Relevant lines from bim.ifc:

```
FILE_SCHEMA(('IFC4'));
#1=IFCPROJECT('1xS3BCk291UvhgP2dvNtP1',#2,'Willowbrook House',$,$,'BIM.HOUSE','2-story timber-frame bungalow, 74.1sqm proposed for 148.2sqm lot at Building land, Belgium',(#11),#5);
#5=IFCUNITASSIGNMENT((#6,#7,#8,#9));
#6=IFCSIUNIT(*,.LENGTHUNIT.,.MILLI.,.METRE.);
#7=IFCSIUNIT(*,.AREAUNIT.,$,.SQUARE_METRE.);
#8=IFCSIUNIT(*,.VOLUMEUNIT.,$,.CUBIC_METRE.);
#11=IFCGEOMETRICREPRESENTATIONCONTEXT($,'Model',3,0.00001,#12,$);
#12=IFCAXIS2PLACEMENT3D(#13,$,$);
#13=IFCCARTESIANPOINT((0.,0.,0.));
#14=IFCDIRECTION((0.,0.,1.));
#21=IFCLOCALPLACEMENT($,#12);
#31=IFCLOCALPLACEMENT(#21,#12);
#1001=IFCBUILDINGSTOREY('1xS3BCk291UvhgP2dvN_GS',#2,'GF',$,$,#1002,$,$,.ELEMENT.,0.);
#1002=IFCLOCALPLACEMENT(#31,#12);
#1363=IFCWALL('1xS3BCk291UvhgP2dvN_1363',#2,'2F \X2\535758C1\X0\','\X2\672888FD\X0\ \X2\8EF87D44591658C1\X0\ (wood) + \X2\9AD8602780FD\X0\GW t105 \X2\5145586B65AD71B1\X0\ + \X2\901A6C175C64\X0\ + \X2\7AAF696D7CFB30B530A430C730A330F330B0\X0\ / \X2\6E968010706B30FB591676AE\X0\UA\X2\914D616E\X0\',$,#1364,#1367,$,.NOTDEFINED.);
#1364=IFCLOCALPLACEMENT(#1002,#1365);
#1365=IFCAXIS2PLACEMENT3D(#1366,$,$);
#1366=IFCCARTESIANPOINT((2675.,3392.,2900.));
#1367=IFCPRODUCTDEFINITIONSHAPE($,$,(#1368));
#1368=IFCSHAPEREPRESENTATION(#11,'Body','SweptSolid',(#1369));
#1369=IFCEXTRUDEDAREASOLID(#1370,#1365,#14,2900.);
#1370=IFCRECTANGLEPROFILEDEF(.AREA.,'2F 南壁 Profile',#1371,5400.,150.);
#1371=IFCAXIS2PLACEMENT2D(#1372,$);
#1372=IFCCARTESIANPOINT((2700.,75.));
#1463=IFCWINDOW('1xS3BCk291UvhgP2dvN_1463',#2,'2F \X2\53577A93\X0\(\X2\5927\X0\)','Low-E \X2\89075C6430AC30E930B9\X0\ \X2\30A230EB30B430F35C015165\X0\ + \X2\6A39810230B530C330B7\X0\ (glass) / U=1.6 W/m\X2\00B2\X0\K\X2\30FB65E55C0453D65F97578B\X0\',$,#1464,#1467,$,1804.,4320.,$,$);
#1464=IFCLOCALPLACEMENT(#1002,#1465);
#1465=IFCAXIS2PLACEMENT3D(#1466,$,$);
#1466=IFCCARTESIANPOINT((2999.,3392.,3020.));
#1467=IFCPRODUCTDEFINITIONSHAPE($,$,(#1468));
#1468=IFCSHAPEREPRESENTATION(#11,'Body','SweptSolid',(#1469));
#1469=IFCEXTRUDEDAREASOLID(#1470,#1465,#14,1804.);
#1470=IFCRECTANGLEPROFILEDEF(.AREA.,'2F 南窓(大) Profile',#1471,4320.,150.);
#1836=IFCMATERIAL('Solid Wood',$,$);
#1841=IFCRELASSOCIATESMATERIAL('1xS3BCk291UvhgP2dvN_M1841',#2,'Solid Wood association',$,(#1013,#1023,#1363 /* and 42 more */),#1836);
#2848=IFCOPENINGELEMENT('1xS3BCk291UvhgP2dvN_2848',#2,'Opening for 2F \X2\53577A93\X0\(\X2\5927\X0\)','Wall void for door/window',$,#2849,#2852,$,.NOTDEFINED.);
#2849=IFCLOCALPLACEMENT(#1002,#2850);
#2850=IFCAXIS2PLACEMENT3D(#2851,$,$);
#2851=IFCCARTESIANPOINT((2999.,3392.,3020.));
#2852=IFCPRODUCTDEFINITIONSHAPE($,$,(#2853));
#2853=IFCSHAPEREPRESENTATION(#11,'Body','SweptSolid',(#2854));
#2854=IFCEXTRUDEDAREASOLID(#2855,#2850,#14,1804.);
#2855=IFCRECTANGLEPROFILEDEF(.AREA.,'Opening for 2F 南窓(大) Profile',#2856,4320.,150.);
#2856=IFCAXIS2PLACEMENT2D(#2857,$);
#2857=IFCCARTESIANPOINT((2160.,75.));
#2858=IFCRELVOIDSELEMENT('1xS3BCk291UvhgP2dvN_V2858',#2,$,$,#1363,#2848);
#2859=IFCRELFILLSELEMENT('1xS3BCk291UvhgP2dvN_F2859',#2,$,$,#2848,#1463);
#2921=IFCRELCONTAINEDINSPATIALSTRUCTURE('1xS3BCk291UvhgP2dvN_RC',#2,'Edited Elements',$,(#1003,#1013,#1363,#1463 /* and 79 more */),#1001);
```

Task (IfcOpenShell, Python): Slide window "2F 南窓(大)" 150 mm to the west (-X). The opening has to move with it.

```python
import ifcopenshell
import ifcopenshell.api.geometry
import ifcopenshell.util.placement
import ifcopenshell.util.unit

model = ifcopenshell.open("bim.ifc")
unit_scale = ifcopenshell.util.unit.calculate_unit_scale(model)

window = model.by_guid("1xS3BCk291UvhgP2dvN_1463")
opening = window.FillsVoids[0].RelatingOpeningElement
wall = opening.VoidsElements[0].RelatingBuildingElement

wall_matrix = ifcopenshell.util.placement.get_local_placement(wall.ObjectPlacement)
shift = wall_matrix[:3, 0] * -0.15 / unit_scale
before = ifcopenshell.util.placement.get_local_placement(window.ObjectPlacement)[:3, 3].copy()

# The window is not placed relative to its opening, so move both.
for product in (opening, window):
    matrix = ifcopenshell.util.placement.get_local_placement(product.ObjectPlacement)
    matrix[:3, 3] += shift
    ifcopenshell.api.geometry.edit_object_placement(model, product=product, matrix=matrix, is_si=False)

after = ifcopenshell.util.placement.get_local_placement(window.ObjectPlacement)[:3, 3]
print("window moved by", (after - before).round(3) + 0.0)

model.write("bim_edited.ifc")
```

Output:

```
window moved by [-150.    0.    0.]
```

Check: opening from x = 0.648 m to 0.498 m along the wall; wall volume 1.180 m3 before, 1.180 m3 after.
